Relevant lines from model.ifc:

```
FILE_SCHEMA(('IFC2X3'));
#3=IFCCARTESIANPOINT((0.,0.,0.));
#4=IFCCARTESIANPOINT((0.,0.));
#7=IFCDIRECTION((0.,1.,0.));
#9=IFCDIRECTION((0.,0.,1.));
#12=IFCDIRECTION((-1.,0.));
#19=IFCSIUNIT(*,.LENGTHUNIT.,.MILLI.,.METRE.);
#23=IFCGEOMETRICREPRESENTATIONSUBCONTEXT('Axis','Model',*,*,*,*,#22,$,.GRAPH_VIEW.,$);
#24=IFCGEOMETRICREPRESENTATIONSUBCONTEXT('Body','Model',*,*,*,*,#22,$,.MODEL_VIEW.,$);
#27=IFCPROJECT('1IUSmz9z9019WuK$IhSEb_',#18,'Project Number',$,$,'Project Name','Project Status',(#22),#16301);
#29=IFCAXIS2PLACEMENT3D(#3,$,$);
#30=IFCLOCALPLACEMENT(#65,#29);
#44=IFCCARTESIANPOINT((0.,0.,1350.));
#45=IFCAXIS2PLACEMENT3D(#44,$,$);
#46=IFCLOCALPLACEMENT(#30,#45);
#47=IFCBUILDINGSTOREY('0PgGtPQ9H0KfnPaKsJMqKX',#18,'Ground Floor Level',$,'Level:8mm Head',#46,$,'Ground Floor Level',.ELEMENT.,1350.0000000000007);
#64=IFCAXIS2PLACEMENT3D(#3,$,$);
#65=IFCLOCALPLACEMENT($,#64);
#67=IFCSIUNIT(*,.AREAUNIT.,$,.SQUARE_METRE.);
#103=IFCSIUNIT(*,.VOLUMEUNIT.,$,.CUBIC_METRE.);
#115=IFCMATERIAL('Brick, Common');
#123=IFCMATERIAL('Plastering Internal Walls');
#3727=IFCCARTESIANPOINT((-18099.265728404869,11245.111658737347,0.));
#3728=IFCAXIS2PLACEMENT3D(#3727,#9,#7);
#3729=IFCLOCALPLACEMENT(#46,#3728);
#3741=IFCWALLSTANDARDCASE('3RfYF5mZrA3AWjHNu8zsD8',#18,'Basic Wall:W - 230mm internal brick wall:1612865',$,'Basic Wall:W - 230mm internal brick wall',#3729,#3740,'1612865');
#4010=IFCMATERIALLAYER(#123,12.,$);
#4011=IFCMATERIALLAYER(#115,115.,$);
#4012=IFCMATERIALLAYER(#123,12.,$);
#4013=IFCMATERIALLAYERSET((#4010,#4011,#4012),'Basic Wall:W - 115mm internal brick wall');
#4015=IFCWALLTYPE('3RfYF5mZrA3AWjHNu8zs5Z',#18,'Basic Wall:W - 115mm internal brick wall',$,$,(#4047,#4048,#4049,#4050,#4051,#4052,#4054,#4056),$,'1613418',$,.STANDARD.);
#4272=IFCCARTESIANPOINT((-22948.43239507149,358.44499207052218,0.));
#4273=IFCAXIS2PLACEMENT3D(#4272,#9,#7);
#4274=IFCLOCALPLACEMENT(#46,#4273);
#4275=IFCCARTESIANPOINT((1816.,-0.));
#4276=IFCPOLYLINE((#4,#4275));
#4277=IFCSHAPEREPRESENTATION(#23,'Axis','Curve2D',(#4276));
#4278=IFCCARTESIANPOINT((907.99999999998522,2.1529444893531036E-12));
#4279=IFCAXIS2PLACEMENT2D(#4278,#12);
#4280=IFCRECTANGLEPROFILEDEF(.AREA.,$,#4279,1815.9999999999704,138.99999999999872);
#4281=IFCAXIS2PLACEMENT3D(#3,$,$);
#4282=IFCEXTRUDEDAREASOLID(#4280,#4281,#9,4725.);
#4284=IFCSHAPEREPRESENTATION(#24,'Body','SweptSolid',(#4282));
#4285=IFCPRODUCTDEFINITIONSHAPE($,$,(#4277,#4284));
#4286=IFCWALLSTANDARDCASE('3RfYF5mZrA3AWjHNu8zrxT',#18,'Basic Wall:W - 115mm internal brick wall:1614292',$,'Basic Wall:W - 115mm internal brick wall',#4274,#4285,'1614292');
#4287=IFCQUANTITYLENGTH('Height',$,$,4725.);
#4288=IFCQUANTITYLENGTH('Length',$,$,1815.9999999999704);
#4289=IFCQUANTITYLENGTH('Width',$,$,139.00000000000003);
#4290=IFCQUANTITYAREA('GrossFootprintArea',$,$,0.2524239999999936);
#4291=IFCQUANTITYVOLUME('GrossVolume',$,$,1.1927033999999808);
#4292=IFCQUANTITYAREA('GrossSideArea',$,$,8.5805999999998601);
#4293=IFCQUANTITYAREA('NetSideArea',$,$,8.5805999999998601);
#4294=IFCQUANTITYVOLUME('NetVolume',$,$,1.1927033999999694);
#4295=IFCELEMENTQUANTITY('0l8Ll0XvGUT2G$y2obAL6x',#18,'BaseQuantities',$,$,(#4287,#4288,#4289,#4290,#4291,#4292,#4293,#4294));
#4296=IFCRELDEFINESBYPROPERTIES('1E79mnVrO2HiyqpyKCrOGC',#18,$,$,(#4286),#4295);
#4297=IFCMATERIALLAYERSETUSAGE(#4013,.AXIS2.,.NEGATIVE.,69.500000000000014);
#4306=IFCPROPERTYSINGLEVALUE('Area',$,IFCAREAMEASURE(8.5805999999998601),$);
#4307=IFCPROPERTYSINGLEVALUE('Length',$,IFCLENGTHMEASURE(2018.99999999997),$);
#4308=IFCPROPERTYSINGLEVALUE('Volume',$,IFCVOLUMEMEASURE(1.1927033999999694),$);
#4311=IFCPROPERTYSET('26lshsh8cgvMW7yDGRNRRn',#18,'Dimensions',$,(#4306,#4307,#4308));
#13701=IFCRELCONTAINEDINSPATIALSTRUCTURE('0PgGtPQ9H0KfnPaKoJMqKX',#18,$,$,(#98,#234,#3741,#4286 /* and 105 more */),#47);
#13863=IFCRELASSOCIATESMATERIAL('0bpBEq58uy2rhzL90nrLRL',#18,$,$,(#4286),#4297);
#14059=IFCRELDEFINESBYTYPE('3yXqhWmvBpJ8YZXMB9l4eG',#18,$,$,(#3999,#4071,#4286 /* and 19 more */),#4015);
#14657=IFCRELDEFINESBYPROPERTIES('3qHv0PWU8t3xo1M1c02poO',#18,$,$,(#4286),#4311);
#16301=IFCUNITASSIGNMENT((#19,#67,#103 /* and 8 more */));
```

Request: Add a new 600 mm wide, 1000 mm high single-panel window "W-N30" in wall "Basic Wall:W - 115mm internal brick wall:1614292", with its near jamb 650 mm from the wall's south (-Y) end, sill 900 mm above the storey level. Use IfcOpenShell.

```python
import numpy as np
import ifcopenshell
import ifcopenshell.api.feature
import ifcopenshell.api.geometry
import ifcopenshell.api.pset
import ifcopenshell.api.root
import ifcopenshell.api.spatial
import ifcopenshell.api.type
import ifcopenshell.geom
import ifcopenshell.util.element
import ifcopenshell.util.placement
import ifcopenshell.util.representation
import ifcopenshell.util.shape
import ifcopenshell.util.unit

model = ifcopenshell.open("model.ifc")
unit_scale = ifcopenshell.util.unit.calculate_unit_scale(model)
area_scale = ifcopenshell.util.unit.calculate_unit_scale(model, "AREAUNIT")
volume_scale = ifcopenshell.util.unit.calculate_unit_scale(model, "VOLUMEUNIT")
settings = ifcopenshell.geom.settings()


def volume(element):
    """Net volume in cubic metres, openings subtracted."""
    shape = ifcopenshell.geom.create_shape(settings, element)
    return ifcopenshell.util.shape.get_volume(shape.geometry)


wall = model.by_guid("3RfYF5mZrA3AWjHNu8zrxT")
storey = ifcopenshell.util.element.get_container(wall, ifc_class="IfcBuildingStorey")
context = ifcopenshell.util.representation.get_context(model, "Model", "Body", "MODEL_VIEW")
before = volume(wall)

width, height, from_end, sill = 0.6, 1, 0.65, 0.9  # metres

# The wall runs along its own X axis, and the end named is its -X end.
wall_shape = ifcopenshell.geom.create_shape(settings, wall)
x, y, z = ifcopenshell.util.shape.get_vertices(wall_shape.geometry).T
start = x.min() + from_end
face, thickness = float(y.min()), float(y.max() - y.min())
wall_matrix = ifcopenshell.util.placement.get_local_placement(wall.ObjectPlacement)
level = ifcopenshell.util.placement.get_local_placement(storey.ObjectPlacement)[2, 3]


def in_wall(x, y):
    """Placement at x, y metres in the wall's axes, at sill height."""
    matrix = wall_matrix.copy()
    matrix[:, 3] = wall_matrix @ np.array([x / unit_scale, y / unit_scale, 0.0, 1.0])
    matrix[2, 3] = level + sill / unit_scale
    return matrix


# Opening: a box that overshoots both wall faces by 50 mm.
opening = ifcopenshell.api.root.create_entity(model, ifc_class="IfcOpeningElement")
box = ifcopenshell.api.geometry.add_wall_representation(
    model, context=context, length=width, height=height, thickness=thickness + 0.1
)
ifcopenshell.api.geometry.assign_representation(model, product=opening, representation=box)
ifcopenshell.api.geometry.edit_object_placement(model, product=opening, matrix=in_wall(start, face - 0.05), is_si=False)
ifcopenshell.api.feature.add_feature(model, feature=opening, element=wall)

window = ifcopenshell.api.root.create_entity(model, ifc_class="IfcWindow", name="W-N30")
window.OverallWidth, window.OverallHeight = width / unit_scale, height / unit_scale
body = ifcopenshell.api.geometry.add_window_representation(
    model,
    context=context,
    overall_width=window.OverallWidth,
    overall_height=window.OverallHeight,
    partition_type="SINGLE_PANEL",
)
ifcopenshell.api.geometry.assign_representation(model, product=window, representation=body)
ifcopenshell.api.spatial.assign_container(model, products=[window], relating_structure=storey)
fills = ifcopenshell.api.feature.add_filling(model, opening=opening, element=window)
fills.OwnerHistory = window.OwnerHistory  # required in IFC2X3

# IFC2X3 keeps the operation on the window style.
style = ifcopenshell.api.root.create_entity(model, ifc_class="IfcWindowStyle", name="W-N30")
style.OperationType, style.ConstructionType = "SINGLE_PANEL", "NOTDEFINED"
style.ParameterTakesPrecedence = style.Sizeable = False
ifcopenshell.api.type.assign_type(model, related_objects=[window], relating_type=style)

# Centre the window in the wall's thickness.
ifcopenshell.api.geometry.edit_object_placement(model, product=window, matrix=in_wall(start, face), is_si=False)
window_shape = ifcopenshell.geom.create_shape(settings, window)
depth = ifcopenshell.util.shape.get_vertices(window_shape.geometry)[:, 1]
offset = face + thickness / 2 - (depth.min() + depth.max()) / 2
ifcopenshell.api.geometry.edit_object_placement(model, product=window, matrix=in_wall(start, offset), is_si=False)

after = volume(wall)

# Update the wall's stored quantities.
qto = model.by_id(ifcopenshell.util.element.get_pset(wall, "BaseQuantities", should_inherit=False)["id"])
ifcopenshell.api.pset.edit_qto(model, qto=qto, properties={
    "NetSideArea": after / thickness / area_scale,
    "NetVolume": after / volume_scale,
})
pset = model.by_id(ifcopenshell.util.element.get_pset(wall, "Dimensions", should_inherit=False)["id"])
ifcopenshell.api.pset.edit_pset(model, pset=pset, properties={
    "Area": model.create_entity("IfcAreaMeasure", after / thickness / area_scale),
    "Volume": model.create_entity("IfcVolumeMeasure", after / volume_scale),
})

print(f"wall volume {before:.3f} -> {after:.3f} m3")

model.write("model-out.ifc")
```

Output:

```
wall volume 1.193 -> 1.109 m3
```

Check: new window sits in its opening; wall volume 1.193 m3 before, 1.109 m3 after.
